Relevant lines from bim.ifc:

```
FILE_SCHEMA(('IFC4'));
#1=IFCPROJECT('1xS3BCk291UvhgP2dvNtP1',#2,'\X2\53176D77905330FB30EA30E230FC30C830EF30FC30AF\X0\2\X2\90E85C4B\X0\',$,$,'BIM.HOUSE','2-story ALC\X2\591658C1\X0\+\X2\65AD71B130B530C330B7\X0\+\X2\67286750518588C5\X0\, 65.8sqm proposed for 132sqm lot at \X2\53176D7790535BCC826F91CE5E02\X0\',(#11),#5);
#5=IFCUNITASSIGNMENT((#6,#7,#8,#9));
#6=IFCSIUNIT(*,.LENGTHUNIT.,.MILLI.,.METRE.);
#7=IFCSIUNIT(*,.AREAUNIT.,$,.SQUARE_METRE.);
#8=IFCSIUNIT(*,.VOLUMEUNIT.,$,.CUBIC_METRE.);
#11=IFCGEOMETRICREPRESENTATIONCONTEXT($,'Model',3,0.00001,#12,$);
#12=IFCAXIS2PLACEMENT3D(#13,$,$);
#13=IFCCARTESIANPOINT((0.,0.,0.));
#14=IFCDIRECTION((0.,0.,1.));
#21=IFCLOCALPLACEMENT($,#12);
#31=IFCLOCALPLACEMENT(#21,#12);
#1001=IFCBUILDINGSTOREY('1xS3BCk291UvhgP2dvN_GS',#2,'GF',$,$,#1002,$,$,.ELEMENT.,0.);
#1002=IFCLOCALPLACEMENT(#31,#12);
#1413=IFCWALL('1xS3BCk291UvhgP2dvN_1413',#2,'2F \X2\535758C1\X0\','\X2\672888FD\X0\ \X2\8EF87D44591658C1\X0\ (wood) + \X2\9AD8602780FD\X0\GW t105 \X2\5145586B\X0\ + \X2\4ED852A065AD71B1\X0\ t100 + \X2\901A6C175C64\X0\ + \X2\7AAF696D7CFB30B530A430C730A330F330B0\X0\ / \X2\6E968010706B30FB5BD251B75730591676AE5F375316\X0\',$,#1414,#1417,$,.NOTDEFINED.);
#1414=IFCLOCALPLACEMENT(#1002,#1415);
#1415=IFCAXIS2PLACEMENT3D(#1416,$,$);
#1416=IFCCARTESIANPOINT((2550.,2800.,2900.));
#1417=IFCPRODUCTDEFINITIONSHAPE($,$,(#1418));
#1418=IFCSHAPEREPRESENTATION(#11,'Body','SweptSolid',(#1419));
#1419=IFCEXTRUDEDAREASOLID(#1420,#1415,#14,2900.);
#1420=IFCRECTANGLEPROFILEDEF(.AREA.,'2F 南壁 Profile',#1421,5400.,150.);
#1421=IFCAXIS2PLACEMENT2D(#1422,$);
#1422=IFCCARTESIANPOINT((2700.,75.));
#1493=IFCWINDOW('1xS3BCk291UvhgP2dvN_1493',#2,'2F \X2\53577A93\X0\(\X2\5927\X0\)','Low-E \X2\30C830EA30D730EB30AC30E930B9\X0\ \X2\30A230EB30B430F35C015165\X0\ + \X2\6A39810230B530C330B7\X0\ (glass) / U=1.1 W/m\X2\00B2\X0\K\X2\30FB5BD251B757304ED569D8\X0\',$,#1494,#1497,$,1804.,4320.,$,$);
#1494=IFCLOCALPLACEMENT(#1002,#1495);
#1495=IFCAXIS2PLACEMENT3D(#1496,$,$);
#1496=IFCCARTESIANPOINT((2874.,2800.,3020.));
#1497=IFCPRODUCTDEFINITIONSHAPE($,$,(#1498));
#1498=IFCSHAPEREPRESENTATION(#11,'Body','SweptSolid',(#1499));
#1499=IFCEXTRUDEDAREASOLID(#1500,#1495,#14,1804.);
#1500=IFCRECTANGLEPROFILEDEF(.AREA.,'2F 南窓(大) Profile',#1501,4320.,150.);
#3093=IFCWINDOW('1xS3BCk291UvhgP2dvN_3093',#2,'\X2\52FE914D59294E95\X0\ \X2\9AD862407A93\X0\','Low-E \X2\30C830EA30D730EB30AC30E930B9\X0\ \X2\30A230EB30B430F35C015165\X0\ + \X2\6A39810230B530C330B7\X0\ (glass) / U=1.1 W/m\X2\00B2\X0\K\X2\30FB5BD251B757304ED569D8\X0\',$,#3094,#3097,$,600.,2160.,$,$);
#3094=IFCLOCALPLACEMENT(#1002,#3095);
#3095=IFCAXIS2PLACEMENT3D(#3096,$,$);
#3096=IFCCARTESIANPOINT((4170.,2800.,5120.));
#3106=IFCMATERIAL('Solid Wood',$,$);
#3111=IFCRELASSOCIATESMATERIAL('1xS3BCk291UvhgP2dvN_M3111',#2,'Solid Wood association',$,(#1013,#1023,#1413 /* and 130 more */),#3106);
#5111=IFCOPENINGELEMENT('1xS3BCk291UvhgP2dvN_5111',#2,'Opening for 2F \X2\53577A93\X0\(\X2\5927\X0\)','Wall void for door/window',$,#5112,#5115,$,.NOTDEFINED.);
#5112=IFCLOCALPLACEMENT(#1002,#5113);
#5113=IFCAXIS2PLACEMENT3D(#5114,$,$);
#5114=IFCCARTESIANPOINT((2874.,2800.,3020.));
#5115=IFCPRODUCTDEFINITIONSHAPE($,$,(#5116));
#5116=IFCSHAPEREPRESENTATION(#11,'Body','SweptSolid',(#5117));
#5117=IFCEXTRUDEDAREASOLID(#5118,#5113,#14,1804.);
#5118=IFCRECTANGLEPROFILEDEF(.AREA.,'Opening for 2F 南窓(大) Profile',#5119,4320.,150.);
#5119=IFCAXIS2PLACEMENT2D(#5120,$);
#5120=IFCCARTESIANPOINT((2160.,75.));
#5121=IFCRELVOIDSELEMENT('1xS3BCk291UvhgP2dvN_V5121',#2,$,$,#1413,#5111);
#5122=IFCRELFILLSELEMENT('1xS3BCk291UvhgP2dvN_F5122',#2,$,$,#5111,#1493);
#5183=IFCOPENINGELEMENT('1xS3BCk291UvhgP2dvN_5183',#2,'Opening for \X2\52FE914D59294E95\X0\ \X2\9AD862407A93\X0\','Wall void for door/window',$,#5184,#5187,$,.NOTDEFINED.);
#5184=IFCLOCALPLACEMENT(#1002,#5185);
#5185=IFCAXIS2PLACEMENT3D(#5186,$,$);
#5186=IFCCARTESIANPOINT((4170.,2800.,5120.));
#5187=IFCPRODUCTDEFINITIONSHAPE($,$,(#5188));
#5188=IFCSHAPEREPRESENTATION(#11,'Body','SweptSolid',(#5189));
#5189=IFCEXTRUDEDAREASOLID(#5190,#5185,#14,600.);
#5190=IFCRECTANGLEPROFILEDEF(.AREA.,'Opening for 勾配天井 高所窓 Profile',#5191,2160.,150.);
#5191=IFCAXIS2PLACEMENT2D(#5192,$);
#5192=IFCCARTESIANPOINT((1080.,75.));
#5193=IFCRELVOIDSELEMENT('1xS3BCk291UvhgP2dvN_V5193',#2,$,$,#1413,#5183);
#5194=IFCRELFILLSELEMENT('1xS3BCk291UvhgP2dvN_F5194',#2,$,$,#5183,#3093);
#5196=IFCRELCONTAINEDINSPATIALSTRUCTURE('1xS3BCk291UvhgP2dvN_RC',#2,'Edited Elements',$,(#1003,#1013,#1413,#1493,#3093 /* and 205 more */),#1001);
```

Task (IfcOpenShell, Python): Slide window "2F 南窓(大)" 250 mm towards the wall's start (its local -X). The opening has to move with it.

```python
import ifcopenshell
import ifcopenshell.api.geometry
import ifcopenshell.util.placement

model = ifcopenshell.open("bim.ifc")

window = model.by_id(1493)
opening = window.FillsVoids[0].RelatingOpeningElement
wall = opening.VoidsElements[0].RelatingBuildingElement

wall_matrix = ifcopenshell.util.placement.get_local_placement(wall.ObjectPlacement)
shift = wall_matrix[:3, 0] * -250.0
before = ifcopenshell.util.placement.get_local_placement(window.ObjectPlacement)[:3, 3].copy()

# The window is not placed relative to its opening, so move both.
for product in (opening, window):
    matrix = ifcopenshell.util.placement.get_local_placement(product.ObjectPlacement)
    matrix[:3, 3] += shift
    ifcopenshell.api.geometry.edit_object_placement(model, product=product, matrix=matrix, is_si=False)

after = ifcopenshell.util.placement.get_local_placement(window.ObjectPlacement)[:3, 3]
print("window moved by", (after - before).round(3) + 0.0)

model.write("bim_edited.ifc")
```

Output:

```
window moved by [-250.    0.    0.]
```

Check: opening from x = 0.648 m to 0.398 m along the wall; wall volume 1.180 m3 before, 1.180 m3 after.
